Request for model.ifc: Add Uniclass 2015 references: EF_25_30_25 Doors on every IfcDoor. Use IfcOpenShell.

First a look at what the model holds.

```python
import ifcopenshell

model = ifcopenshell.open("model.ifc")
print(model.schema)
print("classifications:", [c.Name for c in model.by_type("IfcClassification")])
for ifc_class in ("IfcDoor", "IfcRoof", "IfcStair", "IfcWall", "IfcWindow"):
    print(ifc_class, len(model.by_type(ifc_class)))
```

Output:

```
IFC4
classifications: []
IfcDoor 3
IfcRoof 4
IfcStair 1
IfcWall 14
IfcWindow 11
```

```python
import ifcopenshell
import ifcopenshell.api.classification

model = ifcopenshell.open("model.ifc")

system = ifcopenshell.api.classification.add_classification(model, classification="Uniclass 2015")

codes = {
    "IfcDoor": ("EF_25_30_25", "Doors"),
}
for ifc_class, (code, name) in codes.items():
    products = model.by_type(ifc_class)
    ifcopenshell.api.classification.add_reference(
        model, products=products, classification=system, identification=code, name=name
    )
    print(code, len(products))

model.write("model_v2.ifc")
```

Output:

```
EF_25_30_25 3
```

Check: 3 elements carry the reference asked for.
